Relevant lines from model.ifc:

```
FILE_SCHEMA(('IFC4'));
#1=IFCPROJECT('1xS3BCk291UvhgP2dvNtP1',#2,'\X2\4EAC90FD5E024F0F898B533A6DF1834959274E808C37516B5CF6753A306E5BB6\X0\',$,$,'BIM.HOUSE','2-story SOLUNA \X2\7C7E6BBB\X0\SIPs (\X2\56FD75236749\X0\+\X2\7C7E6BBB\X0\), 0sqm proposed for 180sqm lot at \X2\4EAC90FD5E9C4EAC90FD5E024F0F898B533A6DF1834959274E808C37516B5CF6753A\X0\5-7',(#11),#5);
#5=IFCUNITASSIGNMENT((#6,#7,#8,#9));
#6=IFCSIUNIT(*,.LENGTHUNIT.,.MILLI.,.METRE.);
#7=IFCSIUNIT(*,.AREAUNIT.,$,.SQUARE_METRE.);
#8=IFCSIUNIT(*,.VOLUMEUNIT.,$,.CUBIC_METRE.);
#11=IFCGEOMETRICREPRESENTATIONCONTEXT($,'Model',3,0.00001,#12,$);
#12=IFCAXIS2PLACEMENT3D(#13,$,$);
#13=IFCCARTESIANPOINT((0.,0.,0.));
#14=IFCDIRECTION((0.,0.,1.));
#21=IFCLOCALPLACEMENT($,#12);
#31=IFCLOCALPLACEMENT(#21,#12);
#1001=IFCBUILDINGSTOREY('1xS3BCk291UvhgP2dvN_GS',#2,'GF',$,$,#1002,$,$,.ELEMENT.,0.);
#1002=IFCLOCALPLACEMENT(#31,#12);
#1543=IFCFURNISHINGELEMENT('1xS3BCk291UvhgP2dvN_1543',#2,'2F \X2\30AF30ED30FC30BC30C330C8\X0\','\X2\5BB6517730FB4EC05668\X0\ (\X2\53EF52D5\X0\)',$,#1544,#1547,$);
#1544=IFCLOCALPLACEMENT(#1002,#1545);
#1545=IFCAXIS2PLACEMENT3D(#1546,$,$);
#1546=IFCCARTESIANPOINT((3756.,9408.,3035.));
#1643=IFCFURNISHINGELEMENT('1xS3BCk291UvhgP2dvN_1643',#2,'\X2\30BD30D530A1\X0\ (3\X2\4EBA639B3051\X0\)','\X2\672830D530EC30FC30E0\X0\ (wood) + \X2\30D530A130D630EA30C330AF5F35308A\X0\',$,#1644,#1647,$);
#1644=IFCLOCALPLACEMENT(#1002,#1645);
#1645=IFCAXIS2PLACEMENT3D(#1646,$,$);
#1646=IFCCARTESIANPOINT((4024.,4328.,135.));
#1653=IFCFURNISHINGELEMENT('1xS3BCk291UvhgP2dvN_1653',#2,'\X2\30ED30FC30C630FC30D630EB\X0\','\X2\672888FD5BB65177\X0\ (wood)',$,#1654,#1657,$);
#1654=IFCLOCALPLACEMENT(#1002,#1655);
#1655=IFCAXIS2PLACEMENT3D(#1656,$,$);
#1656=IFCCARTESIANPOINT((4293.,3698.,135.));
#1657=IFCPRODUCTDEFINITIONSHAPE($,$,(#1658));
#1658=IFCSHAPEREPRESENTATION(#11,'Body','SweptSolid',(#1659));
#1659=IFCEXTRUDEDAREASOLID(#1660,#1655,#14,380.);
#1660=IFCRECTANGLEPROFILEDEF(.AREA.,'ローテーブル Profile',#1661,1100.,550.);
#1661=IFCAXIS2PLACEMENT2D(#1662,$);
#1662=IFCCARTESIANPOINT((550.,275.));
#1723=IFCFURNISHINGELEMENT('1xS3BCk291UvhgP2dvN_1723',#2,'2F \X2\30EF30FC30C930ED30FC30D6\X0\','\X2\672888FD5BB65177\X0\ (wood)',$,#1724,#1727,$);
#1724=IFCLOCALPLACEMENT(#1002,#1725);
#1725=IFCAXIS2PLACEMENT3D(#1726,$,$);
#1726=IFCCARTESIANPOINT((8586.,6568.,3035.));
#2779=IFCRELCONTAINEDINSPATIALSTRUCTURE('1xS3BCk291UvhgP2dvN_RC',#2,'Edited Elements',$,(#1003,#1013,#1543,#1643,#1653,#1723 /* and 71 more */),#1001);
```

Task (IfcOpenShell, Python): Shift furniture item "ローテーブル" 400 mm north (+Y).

```python
import ifcopenshell
import ifcopenshell.api.geometry
import ifcopenshell.util.placement
import ifcopenshell.util.unit

model = ifcopenshell.open("model.ifc")
unit_scale = ifcopenshell.util.unit.calculate_unit_scale(model)

item = model.by_id(1653)
matrix = ifcopenshell.util.placement.get_local_placement(item.ObjectPlacement)
matrix[1, 3] += 0.4 / unit_scale
ifcopenshell.api.geometry.edit_object_placement(model, product=item, matrix=matrix, is_si=False)

print(ifcopenshell.util.placement.get_local_placement(item.ObjectPlacement).round(3) + 0.0)

model.write("model-out.ifc")
```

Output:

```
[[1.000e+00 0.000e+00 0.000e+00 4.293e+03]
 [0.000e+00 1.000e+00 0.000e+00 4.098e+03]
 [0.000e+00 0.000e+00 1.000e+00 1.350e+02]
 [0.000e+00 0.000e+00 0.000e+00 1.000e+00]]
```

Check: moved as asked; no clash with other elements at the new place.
